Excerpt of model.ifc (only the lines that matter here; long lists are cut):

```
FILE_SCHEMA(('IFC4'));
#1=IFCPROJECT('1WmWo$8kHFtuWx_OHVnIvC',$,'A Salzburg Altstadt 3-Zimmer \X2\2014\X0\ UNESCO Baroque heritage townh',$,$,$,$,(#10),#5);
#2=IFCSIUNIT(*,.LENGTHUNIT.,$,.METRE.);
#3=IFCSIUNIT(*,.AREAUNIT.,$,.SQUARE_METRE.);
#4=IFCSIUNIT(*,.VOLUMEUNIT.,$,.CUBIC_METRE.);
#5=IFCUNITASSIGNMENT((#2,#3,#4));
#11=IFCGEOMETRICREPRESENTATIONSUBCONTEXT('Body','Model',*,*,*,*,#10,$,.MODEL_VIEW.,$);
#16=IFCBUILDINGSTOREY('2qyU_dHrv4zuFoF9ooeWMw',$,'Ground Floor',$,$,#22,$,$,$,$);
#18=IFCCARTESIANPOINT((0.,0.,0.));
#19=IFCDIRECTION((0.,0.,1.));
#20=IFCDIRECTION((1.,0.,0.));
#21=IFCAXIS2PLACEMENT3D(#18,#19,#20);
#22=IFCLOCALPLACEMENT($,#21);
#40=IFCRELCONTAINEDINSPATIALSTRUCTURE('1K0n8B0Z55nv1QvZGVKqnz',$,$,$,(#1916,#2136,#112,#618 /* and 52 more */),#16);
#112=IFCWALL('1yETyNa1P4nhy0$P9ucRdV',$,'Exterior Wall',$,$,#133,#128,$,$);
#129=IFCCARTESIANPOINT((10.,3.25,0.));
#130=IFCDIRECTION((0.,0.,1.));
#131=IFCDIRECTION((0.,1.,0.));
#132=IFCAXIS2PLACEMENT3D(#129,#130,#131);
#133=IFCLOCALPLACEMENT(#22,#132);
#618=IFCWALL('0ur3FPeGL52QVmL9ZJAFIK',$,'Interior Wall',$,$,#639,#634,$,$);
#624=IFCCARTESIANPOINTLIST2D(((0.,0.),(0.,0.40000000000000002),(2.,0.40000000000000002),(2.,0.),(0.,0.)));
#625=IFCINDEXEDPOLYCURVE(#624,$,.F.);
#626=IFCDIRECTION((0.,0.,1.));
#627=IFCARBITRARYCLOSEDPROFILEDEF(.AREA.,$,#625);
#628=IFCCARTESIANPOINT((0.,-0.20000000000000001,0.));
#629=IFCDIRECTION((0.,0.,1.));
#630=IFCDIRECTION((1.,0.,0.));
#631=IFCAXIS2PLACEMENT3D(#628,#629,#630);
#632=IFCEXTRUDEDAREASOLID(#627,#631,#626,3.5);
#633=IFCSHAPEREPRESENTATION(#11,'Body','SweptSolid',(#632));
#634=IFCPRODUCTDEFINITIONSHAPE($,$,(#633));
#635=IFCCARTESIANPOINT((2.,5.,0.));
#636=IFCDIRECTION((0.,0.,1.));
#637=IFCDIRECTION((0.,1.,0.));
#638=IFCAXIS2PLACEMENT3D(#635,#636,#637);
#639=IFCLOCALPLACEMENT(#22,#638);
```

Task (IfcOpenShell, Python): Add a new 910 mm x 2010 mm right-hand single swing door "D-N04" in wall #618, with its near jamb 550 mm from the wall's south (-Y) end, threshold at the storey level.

```python
import numpy as np
import ifcopenshell
import ifcopenshell.api.feature
import ifcopenshell.api.geometry
import ifcopenshell.api.root
import ifcopenshell.api.spatial
import ifcopenshell.geom
import ifcopenshell.util.element
import ifcopenshell.util.placement
import ifcopenshell.util.representation
import ifcopenshell.util.shape
import ifcopenshell.util.unit

model = ifcopenshell.open("model.ifc")
unit_scale = ifcopenshell.util.unit.calculate_unit_scale(model)
settings = ifcopenshell.geom.settings()


def volume(element):
    """Net volume in cubic metres, openings subtracted."""
    shape = ifcopenshell.geom.create_shape(settings, element)
    return ifcopenshell.util.shape.get_volume(shape.geometry)


wall = model.by_id(618)
storey = ifcopenshell.util.element.get_container(wall, ifc_class="IfcBuildingStorey")
context = ifcopenshell.util.representation.get_context(model, "Model", "Body", "MODEL_VIEW")
before = volume(wall)

width, height, from_end, sill = 0.91, 2.01, 0.55, 0.0  # metres

# The wall runs along its own X axis, and the end named is its -X end.
wall_shape = ifcopenshell.geom.create_shape(settings, wall)
x, y, z = ifcopenshell.util.shape.get_vertices(wall_shape.geometry).T
start = x.min() + from_end
face, thickness = float(y.min()), float(y.max() - y.min())
wall_matrix = ifcopenshell.util.placement.get_local_placement(wall.ObjectPlacement)
level = ifcopenshell.util.placement.get_local_placement(storey.ObjectPlacement)[2, 3]


def in_wall(x, y):
    """Placement at x, y metres in the wall's axes, at sill height."""
    matrix = wall_matrix.copy()
    matrix[:, 3] = wall_matrix @ np.array([x / unit_scale, y / unit_scale, 0.0, 1.0])
    matrix[2, 3] = level + sill / unit_scale
    return matrix


# Opening: a box that overshoots both wall faces by 50 mm.
opening = ifcopenshell.api.root.create_entity(model, ifc_class="IfcOpeningElement", predefined_type="OPENING")
box = ifcopenshell.api.geometry.add_wall_representation(
    model, context=context, length=width, height=height, thickness=thickness + 0.1
)
ifcopenshell.api.geometry.assign_representation(model, product=opening, representation=box)
ifcopenshell.api.geometry.edit_object_placement(model, product=opening, matrix=in_wall(start, face - 0.05), is_si=False)
ifcopenshell.api.feature.add_feature(model, feature=opening, element=wall)

door = ifcopenshell.api.root.create_entity(model, ifc_class="IfcDoor", name="D-N04", predefined_type="DOOR")
door.OverallWidth, door.OverallHeight = width / unit_scale, height / unit_scale
door.OperationType = "SINGLE_SWING_RIGHT"
body = ifcopenshell.api.geometry.add_door_representation(
    model,
    context=context,
    overall_width=door.OverallWidth,
    overall_height=door.OverallHeight,
    operation_type="SINGLE_SWING_RIGHT",
    lining_properties={"LiningDepth": thickness / unit_scale, "ThresholdDepth": thickness / unit_scale},
)
ifcopenshell.api.geometry.assign_representation(model, product=door, representation=body)
ifcopenshell.api.spatial.assign_container(model, products=[door], relating_structure=storey)
ifcopenshell.api.feature.add_filling(model, opening=opening, element=door)

# The lining spans the wall, so the door starts at the wall face.
ifcopenshell.api.geometry.edit_object_placement(model, product=door, matrix=in_wall(start, face), is_si=False)

after = volume(wall)

print(f"wall volume {before:.3f} -> {after:.3f} m3")

model.write("model-out.ifc")
```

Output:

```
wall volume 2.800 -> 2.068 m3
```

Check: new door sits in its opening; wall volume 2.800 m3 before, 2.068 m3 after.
